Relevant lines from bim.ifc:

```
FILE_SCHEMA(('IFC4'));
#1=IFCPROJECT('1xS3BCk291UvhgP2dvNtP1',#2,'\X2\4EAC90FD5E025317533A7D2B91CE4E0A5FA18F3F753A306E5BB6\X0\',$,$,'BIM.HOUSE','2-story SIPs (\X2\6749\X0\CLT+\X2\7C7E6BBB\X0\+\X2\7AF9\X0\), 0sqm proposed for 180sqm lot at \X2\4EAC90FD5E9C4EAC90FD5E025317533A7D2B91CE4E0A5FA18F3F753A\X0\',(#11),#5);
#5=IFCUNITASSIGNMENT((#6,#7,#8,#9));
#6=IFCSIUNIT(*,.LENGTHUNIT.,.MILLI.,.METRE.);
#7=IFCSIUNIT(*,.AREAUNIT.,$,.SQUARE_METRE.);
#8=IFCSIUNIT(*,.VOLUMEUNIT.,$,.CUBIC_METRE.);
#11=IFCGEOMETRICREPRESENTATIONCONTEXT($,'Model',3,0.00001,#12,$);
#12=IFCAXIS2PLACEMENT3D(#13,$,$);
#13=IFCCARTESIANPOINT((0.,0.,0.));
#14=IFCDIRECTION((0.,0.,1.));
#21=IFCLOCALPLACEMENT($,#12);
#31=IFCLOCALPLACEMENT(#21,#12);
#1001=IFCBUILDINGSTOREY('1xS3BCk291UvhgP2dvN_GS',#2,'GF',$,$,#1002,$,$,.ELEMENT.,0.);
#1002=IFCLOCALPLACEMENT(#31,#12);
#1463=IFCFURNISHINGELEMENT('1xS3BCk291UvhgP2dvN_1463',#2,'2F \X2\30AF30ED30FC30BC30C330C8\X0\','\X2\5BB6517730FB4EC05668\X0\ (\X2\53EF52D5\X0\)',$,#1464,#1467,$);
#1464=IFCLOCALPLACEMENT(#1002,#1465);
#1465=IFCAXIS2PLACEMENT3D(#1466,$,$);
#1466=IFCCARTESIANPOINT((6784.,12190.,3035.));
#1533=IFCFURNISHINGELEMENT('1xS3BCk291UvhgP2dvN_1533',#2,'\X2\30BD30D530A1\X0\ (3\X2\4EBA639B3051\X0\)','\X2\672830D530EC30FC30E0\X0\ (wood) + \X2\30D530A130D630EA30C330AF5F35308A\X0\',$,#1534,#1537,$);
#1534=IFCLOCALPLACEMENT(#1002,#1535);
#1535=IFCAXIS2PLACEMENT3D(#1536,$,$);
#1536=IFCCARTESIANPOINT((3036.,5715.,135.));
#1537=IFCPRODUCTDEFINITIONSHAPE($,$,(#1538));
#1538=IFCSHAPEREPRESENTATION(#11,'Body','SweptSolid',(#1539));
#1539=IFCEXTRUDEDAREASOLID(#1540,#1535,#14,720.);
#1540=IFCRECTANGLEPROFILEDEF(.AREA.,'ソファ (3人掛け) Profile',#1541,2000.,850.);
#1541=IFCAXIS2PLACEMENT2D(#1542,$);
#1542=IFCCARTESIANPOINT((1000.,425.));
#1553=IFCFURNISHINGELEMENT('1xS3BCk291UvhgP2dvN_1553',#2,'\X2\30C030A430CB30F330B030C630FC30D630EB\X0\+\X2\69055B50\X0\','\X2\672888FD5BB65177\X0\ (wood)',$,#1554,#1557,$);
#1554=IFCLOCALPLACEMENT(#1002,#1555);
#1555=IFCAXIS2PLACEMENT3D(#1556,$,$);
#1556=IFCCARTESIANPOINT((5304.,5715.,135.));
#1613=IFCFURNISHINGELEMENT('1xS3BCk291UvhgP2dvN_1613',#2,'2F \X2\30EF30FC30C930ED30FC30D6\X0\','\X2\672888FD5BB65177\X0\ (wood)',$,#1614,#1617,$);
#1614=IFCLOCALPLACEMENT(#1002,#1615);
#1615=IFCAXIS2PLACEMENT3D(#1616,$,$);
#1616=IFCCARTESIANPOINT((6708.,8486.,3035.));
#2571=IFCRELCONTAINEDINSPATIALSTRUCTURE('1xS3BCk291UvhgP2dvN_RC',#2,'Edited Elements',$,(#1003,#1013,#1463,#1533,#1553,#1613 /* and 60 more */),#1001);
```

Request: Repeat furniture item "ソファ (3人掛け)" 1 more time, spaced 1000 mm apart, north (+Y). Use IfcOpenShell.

```python
import numpy as np
import ifcopenshell
import ifcopenshell.api.geometry
import ifcopenshell.api.root
import ifcopenshell.util.element
import ifcopenshell.util.placement
import ifcopenshell.util.unit

model = ifcopenshell.open("bim.ifc")
unit_scale = ifcopenshell.util.unit.calculate_unit_scale(model)


def reuse_history(source, copy):
    """copy_class also copies each property set's owner history, people and application; keep the originals."""
    for rel in copy.IsDefinedBy:
        if rel.is_a("IfcRelDefinesByProperties") and (history := rel.RelatingPropertyDefinition.OwnerHistory):
            rel.RelatingPropertyDefinition.OwnerHistory = source.OwnerHistory
            ifcopenshell.util.element.remove_deep2(model, history)


source = model.by_guid("1xS3BCk291UvhgP2dvN_1533")
base = ifcopenshell.util.placement.get_local_placement(source.ObjectPlacement)
step = np.array([0.0, 1.0, 0.0]) * 1 / unit_scale

for i in range(1, 2):
    copy = ifcopenshell.api.root.copy_class(model, product=source)
    copy.Representation = ifcopenshell.util.element.copy_deep(
        model, source.Representation, exclude=["IfcGeometricRepresentationContext", "IfcRepresentationMap"]
    )
    reuse_history(source, copy)
    matrix = base.copy()
    matrix[:3, 3] += i * step
    print("added at", matrix[:3, 3].round(3) + 0.0)
    ifcopenshell.api.geometry.edit_object_placement(model, product=copy, matrix=matrix, is_si=False)

model.write("bim_edited.ifc")
```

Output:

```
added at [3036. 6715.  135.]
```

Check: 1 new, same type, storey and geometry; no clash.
